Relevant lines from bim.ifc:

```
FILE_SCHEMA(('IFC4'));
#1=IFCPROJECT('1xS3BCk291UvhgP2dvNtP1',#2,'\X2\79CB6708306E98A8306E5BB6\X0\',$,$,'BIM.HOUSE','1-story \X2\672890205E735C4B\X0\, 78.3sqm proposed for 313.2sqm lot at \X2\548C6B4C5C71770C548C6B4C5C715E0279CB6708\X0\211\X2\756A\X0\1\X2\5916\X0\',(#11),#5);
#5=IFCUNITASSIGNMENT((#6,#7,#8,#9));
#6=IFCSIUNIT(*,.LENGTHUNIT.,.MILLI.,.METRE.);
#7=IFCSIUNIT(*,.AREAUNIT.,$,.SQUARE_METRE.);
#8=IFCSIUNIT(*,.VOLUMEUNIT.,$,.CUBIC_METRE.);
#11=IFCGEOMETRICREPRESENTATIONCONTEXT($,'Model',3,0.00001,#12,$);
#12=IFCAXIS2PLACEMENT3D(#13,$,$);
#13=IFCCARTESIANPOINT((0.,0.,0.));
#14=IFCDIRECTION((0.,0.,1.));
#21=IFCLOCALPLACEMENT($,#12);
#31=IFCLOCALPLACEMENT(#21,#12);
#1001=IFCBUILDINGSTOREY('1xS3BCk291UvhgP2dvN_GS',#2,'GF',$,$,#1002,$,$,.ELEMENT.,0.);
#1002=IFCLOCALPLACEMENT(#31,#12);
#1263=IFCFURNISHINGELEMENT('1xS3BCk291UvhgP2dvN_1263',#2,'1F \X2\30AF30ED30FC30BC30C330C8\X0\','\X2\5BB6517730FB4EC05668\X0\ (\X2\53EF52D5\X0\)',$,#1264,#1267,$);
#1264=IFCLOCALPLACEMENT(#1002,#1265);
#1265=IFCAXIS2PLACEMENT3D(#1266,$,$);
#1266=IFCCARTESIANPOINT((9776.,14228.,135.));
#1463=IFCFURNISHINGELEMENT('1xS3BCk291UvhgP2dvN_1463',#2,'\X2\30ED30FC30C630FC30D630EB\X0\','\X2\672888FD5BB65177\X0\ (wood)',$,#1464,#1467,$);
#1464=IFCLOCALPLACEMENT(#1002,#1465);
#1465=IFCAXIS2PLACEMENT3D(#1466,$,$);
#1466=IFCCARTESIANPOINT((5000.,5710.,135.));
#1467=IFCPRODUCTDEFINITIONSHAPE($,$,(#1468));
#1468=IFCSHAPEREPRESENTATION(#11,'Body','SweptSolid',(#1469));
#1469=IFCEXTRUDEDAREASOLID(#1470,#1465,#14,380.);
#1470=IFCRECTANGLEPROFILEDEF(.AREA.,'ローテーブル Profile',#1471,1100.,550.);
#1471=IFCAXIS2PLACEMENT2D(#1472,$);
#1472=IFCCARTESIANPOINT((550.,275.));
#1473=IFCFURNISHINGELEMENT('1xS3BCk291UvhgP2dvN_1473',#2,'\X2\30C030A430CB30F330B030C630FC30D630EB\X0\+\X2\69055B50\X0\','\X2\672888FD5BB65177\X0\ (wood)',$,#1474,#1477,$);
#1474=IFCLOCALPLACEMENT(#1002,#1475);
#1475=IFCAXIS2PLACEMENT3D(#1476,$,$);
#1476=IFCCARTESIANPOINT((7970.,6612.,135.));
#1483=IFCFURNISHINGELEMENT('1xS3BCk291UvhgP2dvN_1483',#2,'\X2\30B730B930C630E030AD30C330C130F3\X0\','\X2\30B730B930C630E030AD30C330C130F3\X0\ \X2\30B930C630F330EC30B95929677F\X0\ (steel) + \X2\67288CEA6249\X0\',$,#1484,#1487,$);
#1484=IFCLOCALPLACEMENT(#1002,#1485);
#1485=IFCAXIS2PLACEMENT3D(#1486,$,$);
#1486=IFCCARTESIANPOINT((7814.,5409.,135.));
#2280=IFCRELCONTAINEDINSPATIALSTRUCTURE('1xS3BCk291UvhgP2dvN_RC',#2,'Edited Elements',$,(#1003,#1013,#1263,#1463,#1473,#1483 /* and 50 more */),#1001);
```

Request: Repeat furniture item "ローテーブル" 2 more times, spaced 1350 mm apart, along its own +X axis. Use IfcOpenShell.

```python
import ifcopenshell
import ifcopenshell.api.geometry
import ifcopenshell.api.root
import ifcopenshell.util.element
import ifcopenshell.util.placement
import ifcopenshell.util.unit

model = ifcopenshell.open("bim.ifc")
unit_scale = ifcopenshell.util.unit.calculate_unit_scale(model)


def reuse_history(source, copy):
    """copy_class also copies each property set's owner history, people and application; keep the originals."""
    for rel in copy.IsDefinedBy:
        if rel.is_a("IfcRelDefinesByProperties") and (history := rel.RelatingPropertyDefinition.OwnerHistory):
            rel.RelatingPropertyDefinition.OwnerHistory = source.OwnerHistory
            ifcopenshell.util.element.remove_deep2(model, history)


source = model.by_guid("1xS3BCk291UvhgP2dvN_1463")
base = ifcopenshell.util.placement.get_local_placement(source.ObjectPlacement)
step = base[:3, 0] * 1.35 / unit_scale

for i in range(1, 3):
    copy = ifcopenshell.api.root.copy_class(model, product=source)
    copy.Representation = ifcopenshell.util.element.copy_deep(
        model, source.Representation, exclude=["IfcGeometricRepresentationContext", "IfcRepresentationMap"]
    )
    reuse_history(source, copy)
    matrix = base.copy()
    matrix[:3, 3] += i * step
    print("added at", matrix[:3, 3].round(3) + 0.0)
    ifcopenshell.api.geometry.edit_object_placement(model, product=copy, matrix=matrix, is_si=False)

model.write("bim_edited.ifc")
```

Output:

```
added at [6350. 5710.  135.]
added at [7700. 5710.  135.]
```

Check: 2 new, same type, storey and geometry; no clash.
